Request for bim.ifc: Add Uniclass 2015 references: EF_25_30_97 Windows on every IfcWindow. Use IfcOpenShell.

First a look at what the model holds.

```python
import ifcopenshell

model = ifcopenshell.open("bim.ifc")
print(model.schema)
print("classifications:", [c.Name for c in model.by_type("IfcClassification")])
for ifc_class in ("IfcDoor", "IfcRoof", "IfcStair", "IfcWall", "IfcWindow"):
    print(ifc_class, len(model.by_type(ifc_class)))
```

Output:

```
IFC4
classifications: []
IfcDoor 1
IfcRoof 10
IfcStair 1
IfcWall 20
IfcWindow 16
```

```python
import ifcopenshell
import ifcopenshell.api.classification

model = ifcopenshell.open("bim.ifc")

system = ifcopenshell.api.classification.add_classification(model, classification="Uniclass 2015")

codes = {
    "IfcWindow": ("EF_25_30_97", "Windows"),
}
for ifc_class, (code, name) in codes.items():
    products = model.by_type(ifc_class)
    ifcopenshell.api.classification.add_reference(
        model, products=products, classification=system, identification=code, name=name
    )
    print(code, len(products))

model.write("bim_updated.ifc")
```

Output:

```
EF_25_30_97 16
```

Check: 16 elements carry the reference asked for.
